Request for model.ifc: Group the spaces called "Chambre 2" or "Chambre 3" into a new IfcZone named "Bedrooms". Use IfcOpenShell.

First a look at what the model holds.

```python
import ifcopenshell

model = ifcopenshell.open("model.ifc")
print(model.schema)
seen = {}
for space in model.by_type("IfcSpace"):
    seen[space.LongName] = seen.get(space.LongName, 0) + 1
for name, count in sorted(seen.items(), key=str):
    print(count, "x", name)
print("zones:", [z.Name for z in model.by_type("IfcZone")][:20])
```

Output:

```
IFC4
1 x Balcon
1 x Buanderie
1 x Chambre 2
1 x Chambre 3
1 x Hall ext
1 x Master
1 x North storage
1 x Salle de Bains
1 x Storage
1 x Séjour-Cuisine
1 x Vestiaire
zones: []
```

```python
import ifcopenshell
import ifcopenshell.api.group
import ifcopenshell.api.root

model = ifcopenshell.open("model.ifc")

names = {"Chambre 2", "Chambre 3"}
spaces = [s for s in model.by_type("IfcSpace") if s.LongName in names]

zone = ifcopenshell.api.root.create_entity(model, ifc_class="IfcZone", name="Bedrooms")
ifcopenshell.api.group.assign_group(model, products=spaces, group=zone)
print(len(spaces), "spaces in", zone.Name)

model.write("model-out.ifc")
```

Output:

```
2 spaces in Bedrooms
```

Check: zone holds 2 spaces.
